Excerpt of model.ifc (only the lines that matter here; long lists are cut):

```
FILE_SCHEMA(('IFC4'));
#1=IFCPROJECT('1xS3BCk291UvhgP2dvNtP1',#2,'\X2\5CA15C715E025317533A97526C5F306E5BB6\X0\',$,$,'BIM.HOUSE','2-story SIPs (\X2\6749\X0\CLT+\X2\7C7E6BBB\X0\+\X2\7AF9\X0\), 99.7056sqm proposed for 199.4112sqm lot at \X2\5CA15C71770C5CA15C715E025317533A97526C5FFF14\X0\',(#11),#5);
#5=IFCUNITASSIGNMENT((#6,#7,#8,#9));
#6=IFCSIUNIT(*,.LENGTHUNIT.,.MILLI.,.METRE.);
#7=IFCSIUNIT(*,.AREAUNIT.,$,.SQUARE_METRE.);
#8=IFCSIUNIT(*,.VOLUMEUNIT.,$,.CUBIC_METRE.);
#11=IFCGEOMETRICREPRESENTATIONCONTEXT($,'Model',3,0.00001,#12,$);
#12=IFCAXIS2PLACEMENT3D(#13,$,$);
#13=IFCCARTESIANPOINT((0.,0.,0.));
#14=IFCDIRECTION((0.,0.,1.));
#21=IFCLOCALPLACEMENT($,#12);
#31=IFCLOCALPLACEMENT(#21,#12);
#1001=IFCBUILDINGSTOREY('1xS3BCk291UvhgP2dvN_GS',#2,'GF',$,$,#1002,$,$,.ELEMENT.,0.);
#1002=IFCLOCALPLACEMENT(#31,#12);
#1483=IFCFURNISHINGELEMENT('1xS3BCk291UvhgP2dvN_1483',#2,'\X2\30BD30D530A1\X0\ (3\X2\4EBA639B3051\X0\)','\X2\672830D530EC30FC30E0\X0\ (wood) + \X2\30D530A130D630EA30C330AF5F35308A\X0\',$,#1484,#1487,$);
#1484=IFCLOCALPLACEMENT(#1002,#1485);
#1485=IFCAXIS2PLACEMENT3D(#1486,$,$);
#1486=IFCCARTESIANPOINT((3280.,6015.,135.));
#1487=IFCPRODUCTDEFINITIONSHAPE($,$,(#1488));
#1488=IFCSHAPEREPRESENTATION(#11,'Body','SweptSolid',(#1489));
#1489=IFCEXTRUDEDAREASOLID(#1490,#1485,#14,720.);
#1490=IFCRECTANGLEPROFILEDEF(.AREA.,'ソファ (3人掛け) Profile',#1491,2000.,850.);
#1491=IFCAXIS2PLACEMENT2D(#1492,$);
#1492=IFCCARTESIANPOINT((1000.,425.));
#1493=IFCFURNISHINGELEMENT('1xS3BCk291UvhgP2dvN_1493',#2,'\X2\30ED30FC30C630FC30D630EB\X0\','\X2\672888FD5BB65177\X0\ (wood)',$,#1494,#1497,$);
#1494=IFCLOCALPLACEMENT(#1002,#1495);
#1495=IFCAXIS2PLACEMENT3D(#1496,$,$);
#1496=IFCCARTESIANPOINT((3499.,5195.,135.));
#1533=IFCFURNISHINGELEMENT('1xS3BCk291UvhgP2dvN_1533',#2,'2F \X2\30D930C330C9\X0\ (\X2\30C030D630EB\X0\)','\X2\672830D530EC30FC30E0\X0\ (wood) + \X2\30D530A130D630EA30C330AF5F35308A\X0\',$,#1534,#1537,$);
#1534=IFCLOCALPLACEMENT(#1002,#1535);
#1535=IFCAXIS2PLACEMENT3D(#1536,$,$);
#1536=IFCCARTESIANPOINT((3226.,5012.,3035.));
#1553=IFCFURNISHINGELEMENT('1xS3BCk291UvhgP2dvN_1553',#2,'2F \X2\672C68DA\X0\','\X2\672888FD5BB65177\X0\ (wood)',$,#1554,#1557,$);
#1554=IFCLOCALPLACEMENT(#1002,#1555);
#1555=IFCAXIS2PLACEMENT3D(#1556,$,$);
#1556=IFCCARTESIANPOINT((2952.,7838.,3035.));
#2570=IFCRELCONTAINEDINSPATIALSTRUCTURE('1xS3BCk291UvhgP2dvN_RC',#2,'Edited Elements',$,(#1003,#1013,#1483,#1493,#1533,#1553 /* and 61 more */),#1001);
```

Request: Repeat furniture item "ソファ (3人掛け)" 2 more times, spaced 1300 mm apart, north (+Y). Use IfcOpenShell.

```python
import numpy as np
import ifcopenshell
import ifcopenshell.api.geometry
import ifcopenshell.api.root
import ifcopenshell.util.element
import ifcopenshell.util.placement
import ifcopenshell.util.unit

model = ifcopenshell.open("model.ifc")
unit_scale = ifcopenshell.util.unit.calculate_unit_scale(model)


def reuse_history(source, copy):
    """copy_class also copies each property set's owner history, people and application; keep the originals."""
    for rel in copy.IsDefinedBy:
        if rel.is_a("IfcRelDefinesByProperties") and (history := rel.RelatingPropertyDefinition.OwnerHistory):
            rel.RelatingPropertyDefinition.OwnerHistory = source.OwnerHistory
            ifcopenshell.util.element.remove_deep2(model, history)


source = model.by_guid("1xS3BCk291UvhgP2dvN_1483")
base = ifcopenshell.util.placement.get_local_placement(source.ObjectPlacement)
step = np.array([0.0, 1.0, 0.0]) * 1.3 / unit_scale

for i in range(1, 3):
    copy = ifcopenshell.api.root.copy_class(model, product=source)
    copy.Representation = ifcopenshell.util.element.copy_deep(
        model, source.Representation, exclude=["IfcGeometricRepresentationContext", "IfcRepresentationMap"]
    )
    reuse_history(source, copy)
    matrix = base.copy()
    matrix[:3, 3] += i * step
    print("added at", matrix[:3, 3].round(3) + 0.0)
    ifcopenshell.api.geometry.edit_object_placement(model, product=copy, matrix=matrix, is_si=False)

model.write("model_v2.ifc")
```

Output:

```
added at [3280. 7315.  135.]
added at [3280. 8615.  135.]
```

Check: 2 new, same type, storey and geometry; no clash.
